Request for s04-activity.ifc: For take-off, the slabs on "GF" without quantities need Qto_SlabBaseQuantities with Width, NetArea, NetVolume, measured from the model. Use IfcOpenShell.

First a look at what the model holds.

```python
import ifcopenshell
import ifcopenshell.util.element
import ifcopenshell.util.unit

model = ifcopenshell.open("s04-activity.ifc")
print(model.schema)
for unit_type in ("LENGTHUNIT", "AREAUNIT", "VOLUMEUNIT"):
    print(unit_type, ifcopenshell.util.unit.calculate_unit_scale(model, unit_type))
storey = next(s for s in model.by_type("IfcBuildingStorey") if s.Name == "GF")
slabs = [e for e in ifcopenshell.util.element.get_decomposition(storey) if e.is_a("IfcSlab")]
for e in sorted(slabs, key=lambda e: e.id()):
    print(e.id(), e.is_a(), e.Name, list(ifcopenshell.util.element.get_psets(e, qtos_only=True)), sep=" | ")
```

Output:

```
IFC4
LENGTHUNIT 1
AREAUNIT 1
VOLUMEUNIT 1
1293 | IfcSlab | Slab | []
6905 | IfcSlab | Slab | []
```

```python
import ifcopenshell
import ifcopenshell.api.pset
import ifcopenshell.geom
import ifcopenshell.util.element
import ifcopenshell.util.shape
import ifcopenshell.util.unit

model = ifcopenshell.open("s04-activity.ifc")
unit_scale = ifcopenshell.util.unit.calculate_unit_scale(model)
area_scale = ifcopenshell.util.unit.calculate_unit_scale(model, "AREAUNIT")
volume_scale = ifcopenshell.util.unit.calculate_unit_scale(model, "VOLUMEUNIT")
settings = ifcopenshell.geom.settings()

storey = next(s for s in model.by_type("IfcBuildingStorey") if s.Name == "GF")
slabs = [e for e in ifcopenshell.util.element.get_decomposition(storey) if e.is_a("IfcSlab")]

for e in sorted(slabs, key=lambda e: e.id()):
    if ifcopenshell.util.element.get_psets(e, qtos_only=True, should_inherit=False):
        continue
    # Geometry comes back in metres, in the element's own axes.
    shape = ifcopenshell.geom.create_shape(settings, e)
    values = {
        "Width": ifcopenshell.util.shape.get_z(shape.geometry) / unit_scale,
        "NetArea": ifcopenshell.util.shape.get_footprint_area(shape.geometry) / area_scale,
        "NetVolume": ifcopenshell.util.shape.get_volume(shape.geometry) / volume_scale,
    }
    qto = ifcopenshell.api.pset.add_qto(model, product=e, name="Qto_SlabBaseQuantities")
    ifcopenshell.api.pset.edit_qto(model, qto=qto, properties=values)
    print(e.id(), {k: round(v, 3) for k, v in values.items()})

model.write("s04-activity_rev.ifc")
```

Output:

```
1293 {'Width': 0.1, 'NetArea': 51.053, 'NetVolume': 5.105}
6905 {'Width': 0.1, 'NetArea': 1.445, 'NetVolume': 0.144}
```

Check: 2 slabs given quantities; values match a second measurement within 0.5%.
